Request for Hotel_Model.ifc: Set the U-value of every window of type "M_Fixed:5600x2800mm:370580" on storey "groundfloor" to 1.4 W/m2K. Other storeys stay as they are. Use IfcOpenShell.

First a look at what the model holds.

```python
import ifcopenshell
import ifcopenshell.util.element

model = ifcopenshell.open("Hotel_Model.ifc")
print(model.schema)
storey = next(s for s in model.by_type("IfcBuildingStorey") if s.Name == "groundfloor")
windows = [e for e in ifcopenshell.util.element.get_decomposition(storey) if e.is_a("IfcWindow")]
seen = {}
for e in windows:
    element_type = ifcopenshell.util.element.get_type(e)
    key = (element_type.Name if element_type != e and element_type else None, ifcopenshell.util.element.get_pset(e, "Pset_WindowCommon", "ThermalTransmittance"))
    seen[key] = seen.get(key, 0) + 1
for (name, value), count in sorted(seen.items(), key=str):
    print(count, "x", name, "|", value)
```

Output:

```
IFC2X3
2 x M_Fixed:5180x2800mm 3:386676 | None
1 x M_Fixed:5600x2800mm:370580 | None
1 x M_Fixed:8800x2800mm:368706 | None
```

```python
import ifcopenshell
import ifcopenshell.api.pset
import ifcopenshell.util.element

model = ifcopenshell.open("Hotel_Model.ifc")

storey = next(s for s in model.by_type("IfcBuildingStorey") if s.Name == "groundfloor")
windows = [e for e in ifcopenshell.util.element.get_decomposition(storey) if e.is_a("IfcWindow")]

count = 0
for e in windows:
    element_type = ifcopenshell.util.element.get_type(e)
    if element_type in (None, e) or element_type.Name != "M_Fixed:5600x2800mm:370580":
        continue
    # add_pset returns the element's existing set when there is one.
    pset = ifcopenshell.api.pset.add_pset(model, product=e, name="Pset_WindowCommon")
    ifcopenshell.api.pset.edit_pset(model, pset=pset, properties={"ThermalTransmittance": 1.4})
    count += 1

print(count, "windows updated")

model.write("Hotel_Model_rev.ifc")
```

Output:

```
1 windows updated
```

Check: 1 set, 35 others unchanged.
